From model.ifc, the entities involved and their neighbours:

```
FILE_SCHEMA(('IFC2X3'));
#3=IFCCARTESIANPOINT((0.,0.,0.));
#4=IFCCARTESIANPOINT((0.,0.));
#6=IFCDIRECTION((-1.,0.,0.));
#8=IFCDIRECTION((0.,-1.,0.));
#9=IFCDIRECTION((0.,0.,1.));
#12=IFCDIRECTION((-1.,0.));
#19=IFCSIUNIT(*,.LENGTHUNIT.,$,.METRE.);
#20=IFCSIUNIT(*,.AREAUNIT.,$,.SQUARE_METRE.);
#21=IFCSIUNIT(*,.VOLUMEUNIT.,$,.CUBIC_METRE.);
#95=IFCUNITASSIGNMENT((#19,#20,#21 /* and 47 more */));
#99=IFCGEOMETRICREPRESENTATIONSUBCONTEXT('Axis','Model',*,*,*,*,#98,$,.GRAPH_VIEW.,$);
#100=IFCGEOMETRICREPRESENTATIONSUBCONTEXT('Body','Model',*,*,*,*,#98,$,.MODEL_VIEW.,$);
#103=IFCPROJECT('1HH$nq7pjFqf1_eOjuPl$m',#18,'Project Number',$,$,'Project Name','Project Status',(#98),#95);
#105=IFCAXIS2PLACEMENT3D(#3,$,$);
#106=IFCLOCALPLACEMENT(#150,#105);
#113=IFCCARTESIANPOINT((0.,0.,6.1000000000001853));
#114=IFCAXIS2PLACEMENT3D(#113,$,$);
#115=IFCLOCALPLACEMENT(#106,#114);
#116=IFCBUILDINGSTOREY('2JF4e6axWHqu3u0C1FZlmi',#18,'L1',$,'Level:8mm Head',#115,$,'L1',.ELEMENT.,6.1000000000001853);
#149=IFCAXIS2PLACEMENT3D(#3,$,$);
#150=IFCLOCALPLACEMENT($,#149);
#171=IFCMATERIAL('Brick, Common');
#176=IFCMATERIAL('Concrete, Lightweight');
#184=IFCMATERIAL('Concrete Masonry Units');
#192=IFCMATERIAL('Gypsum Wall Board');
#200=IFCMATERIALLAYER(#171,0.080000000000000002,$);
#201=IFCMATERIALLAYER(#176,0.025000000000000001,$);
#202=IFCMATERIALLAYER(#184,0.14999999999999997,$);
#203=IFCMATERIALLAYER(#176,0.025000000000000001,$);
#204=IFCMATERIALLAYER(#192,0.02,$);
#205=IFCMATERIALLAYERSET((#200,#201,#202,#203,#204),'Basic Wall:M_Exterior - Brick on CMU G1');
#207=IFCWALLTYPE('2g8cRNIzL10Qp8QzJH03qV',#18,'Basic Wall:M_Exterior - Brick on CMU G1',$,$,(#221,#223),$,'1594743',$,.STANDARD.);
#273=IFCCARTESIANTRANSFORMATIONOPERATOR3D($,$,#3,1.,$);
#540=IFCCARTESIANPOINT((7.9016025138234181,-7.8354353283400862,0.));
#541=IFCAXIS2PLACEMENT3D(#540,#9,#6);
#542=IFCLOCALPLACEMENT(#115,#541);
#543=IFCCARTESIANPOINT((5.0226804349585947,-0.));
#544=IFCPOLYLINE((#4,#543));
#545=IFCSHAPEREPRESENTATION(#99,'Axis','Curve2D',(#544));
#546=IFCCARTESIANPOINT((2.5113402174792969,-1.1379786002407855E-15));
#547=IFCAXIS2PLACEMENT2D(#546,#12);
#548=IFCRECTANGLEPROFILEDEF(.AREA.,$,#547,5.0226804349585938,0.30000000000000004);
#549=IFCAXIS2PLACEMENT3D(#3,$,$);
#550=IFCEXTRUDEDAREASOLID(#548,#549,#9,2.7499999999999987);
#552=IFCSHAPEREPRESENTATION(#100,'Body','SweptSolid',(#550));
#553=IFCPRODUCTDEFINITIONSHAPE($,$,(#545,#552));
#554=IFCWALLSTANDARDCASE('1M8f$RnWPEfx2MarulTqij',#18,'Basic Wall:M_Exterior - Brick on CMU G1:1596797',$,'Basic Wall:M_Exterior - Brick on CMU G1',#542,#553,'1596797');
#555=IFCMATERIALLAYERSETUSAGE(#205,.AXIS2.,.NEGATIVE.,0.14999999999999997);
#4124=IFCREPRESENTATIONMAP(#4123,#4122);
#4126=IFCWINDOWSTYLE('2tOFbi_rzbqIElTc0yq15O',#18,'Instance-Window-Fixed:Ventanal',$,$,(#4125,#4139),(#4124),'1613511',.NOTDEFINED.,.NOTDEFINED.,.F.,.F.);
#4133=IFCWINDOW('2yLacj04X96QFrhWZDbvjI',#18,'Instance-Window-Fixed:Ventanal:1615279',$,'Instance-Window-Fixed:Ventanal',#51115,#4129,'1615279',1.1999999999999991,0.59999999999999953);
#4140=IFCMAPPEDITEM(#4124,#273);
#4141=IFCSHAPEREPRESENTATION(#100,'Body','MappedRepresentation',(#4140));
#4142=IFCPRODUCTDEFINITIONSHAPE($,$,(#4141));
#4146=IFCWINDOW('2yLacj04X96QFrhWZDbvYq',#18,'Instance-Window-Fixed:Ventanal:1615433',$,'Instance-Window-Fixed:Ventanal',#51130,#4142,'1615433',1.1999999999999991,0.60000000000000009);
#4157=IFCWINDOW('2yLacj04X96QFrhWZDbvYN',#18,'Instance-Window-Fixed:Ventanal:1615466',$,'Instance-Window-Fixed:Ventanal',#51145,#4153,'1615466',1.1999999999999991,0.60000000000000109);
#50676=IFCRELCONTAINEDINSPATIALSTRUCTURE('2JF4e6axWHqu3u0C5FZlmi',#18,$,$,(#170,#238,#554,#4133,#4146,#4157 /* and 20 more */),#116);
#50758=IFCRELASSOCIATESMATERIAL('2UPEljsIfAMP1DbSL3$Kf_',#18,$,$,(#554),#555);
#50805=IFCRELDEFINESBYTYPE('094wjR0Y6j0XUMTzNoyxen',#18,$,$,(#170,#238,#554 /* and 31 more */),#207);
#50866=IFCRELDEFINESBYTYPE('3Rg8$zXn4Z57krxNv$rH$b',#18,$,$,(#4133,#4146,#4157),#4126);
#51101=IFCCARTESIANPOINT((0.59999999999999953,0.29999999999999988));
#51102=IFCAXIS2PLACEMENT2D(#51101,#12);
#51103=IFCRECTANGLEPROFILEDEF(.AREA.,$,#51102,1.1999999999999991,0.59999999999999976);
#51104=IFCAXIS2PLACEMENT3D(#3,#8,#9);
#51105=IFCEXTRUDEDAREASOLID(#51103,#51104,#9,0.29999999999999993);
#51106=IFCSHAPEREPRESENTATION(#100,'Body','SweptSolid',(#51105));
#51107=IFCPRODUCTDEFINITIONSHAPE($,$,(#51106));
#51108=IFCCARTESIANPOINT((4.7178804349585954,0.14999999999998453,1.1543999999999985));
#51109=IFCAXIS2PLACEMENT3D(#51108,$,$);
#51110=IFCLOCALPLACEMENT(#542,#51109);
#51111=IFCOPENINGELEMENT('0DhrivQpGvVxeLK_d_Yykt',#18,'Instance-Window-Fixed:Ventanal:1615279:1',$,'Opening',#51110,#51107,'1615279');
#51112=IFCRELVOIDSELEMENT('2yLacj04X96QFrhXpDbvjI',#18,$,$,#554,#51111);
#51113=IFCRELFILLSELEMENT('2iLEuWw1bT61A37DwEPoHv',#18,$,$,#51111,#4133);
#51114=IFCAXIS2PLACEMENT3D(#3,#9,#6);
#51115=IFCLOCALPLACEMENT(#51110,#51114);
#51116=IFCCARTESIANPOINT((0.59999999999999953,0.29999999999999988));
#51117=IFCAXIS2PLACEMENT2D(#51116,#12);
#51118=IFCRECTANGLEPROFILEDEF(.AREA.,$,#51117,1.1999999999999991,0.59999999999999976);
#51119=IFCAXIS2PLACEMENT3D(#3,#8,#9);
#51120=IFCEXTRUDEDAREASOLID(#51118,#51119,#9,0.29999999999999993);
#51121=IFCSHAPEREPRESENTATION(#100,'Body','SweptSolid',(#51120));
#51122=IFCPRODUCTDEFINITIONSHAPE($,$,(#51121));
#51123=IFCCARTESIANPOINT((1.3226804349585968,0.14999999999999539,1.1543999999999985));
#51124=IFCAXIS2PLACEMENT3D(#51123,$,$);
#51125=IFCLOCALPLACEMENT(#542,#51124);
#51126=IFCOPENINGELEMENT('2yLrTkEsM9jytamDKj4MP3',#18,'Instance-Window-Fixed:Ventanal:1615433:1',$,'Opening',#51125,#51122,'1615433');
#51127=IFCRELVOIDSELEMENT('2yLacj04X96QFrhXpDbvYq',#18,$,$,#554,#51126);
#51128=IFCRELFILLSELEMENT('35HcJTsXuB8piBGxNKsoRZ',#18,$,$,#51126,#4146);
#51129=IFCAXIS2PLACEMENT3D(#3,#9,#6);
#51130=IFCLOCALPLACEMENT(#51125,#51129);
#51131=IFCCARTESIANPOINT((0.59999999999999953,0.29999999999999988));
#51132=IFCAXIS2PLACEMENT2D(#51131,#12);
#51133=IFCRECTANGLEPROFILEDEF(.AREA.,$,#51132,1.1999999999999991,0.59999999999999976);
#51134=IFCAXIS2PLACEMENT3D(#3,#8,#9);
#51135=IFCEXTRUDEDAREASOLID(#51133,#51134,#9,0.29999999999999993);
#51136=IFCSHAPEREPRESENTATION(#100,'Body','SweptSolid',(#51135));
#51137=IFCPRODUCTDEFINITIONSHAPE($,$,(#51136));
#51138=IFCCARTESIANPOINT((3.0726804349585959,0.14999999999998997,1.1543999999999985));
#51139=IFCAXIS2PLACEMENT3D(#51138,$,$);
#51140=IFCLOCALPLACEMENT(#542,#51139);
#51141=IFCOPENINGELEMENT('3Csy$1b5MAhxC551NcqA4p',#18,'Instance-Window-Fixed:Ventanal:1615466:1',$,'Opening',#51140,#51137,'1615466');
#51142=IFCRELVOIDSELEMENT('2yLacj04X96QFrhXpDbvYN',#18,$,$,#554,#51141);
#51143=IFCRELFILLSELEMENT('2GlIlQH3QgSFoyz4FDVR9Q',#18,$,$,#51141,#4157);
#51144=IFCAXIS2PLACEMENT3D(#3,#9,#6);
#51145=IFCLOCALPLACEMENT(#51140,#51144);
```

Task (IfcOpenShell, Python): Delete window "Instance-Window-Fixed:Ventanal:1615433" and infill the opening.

```python
import ifcopenshell
import ifcopenshell.api.feature
import ifcopenshell.api.root
import ifcopenshell.geom
import ifcopenshell.util.shape

model = ifcopenshell.open("model.ifc")
settings = ifcopenshell.geom.settings()


def volume(element):
    """Net volume in cubic metres, openings subtracted."""
    shape = ifcopenshell.geom.create_shape(settings, element)
    return ifcopenshell.util.shape.get_volume(shape.geometry)


window = model.by_id(4146)
opening = window.FillsVoids[0].RelatingOpeningElement
wall = opening.VoidsElements[0].RelatingBuildingElement
before = volume(wall)

ifcopenshell.api.root.remove_product(model, product=window)
ifcopenshell.api.feature.remove_feature(model, feature=opening)

after = volume(wall)

print(f"wall volume {before:.3f} -> {after:.3f} m3")

model.write("model_updated.ifc")
```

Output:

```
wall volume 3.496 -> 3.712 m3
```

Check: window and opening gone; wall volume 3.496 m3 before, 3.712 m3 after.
